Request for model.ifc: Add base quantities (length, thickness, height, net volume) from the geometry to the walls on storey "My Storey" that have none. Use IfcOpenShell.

First a look at what the model holds.

```python
import ifcopenshell
import ifcopenshell.util.element
import ifcopenshell.util.unit

model = ifcopenshell.open("model.ifc")
print(model.schema)
for unit_type in ("LENGTHUNIT", "AREAUNIT", "VOLUMEUNIT"):
    print(unit_type, ifcopenshell.util.unit.calculate_unit_scale(model, unit_type))
storey = next(s for s in model.by_type("IfcBuildingStorey") if s.Name == "My Storey")
walls = [e for e in ifcopenshell.util.element.get_decomposition(storey) if e.is_a("IfcWall")]
for e in sorted(walls, key=lambda e: e.id()):
    print(e.id(), e.is_a(), e.Name, list(ifcopenshell.util.element.get_psets(e, qtos_only=True)), sep=" | ")
```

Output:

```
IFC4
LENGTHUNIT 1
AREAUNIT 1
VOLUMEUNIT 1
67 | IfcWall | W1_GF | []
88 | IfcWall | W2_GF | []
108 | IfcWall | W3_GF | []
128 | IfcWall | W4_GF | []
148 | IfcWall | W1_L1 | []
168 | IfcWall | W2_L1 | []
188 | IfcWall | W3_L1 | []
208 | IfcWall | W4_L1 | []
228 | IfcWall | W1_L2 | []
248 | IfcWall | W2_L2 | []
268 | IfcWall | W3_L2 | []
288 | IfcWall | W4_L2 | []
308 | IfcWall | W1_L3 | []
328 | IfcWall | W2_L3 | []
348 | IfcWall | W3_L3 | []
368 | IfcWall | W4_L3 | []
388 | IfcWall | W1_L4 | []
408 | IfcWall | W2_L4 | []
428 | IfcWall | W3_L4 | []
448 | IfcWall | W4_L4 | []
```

```python
import ifcopenshell
import ifcopenshell.api.pset
import ifcopenshell.geom
import ifcopenshell.util.element
import ifcopenshell.util.shape
import ifcopenshell.util.unit

model = ifcopenshell.open("model.ifc")
unit_scale = ifcopenshell.util.unit.calculate_unit_scale(model)
volume_scale = ifcopenshell.util.unit.calculate_unit_scale(model, "VOLUMEUNIT")
settings = ifcopenshell.geom.settings()

storey = next(s for s in model.by_type("IfcBuildingStorey") if s.Name == "My Storey")
walls = [e for e in ifcopenshell.util.element.get_decomposition(storey) if e.is_a("IfcWall")]

for e in sorted(walls, key=lambda e: e.id()):
    if ifcopenshell.util.element.get_psets(e, qtos_only=True, should_inherit=False):
        continue
    # Geometry comes back in metres, in the element's own axes.
    shape = ifcopenshell.geom.create_shape(settings, e)
    values = {
        "Length": ifcopenshell.util.shape.get_x(shape.geometry) / unit_scale,
        "Width": ifcopenshell.util.shape.get_y(shape.geometry) / unit_scale,
        "Height": ifcopenshell.util.shape.get_z(shape.geometry) / unit_scale,
        "NetVolume": ifcopenshell.util.shape.get_volume(shape.geometry) / volume_scale,
    }
    qto = ifcopenshell.api.pset.add_qto(model, product=e, name="Qto_WallBaseQuantities")
    ifcopenshell.api.pset.edit_qto(model, qto=qto, properties=values)
    print(e.id(), {k: round(v, 3) for k, v in values.items()})

model.write("model_updated.ifc")
```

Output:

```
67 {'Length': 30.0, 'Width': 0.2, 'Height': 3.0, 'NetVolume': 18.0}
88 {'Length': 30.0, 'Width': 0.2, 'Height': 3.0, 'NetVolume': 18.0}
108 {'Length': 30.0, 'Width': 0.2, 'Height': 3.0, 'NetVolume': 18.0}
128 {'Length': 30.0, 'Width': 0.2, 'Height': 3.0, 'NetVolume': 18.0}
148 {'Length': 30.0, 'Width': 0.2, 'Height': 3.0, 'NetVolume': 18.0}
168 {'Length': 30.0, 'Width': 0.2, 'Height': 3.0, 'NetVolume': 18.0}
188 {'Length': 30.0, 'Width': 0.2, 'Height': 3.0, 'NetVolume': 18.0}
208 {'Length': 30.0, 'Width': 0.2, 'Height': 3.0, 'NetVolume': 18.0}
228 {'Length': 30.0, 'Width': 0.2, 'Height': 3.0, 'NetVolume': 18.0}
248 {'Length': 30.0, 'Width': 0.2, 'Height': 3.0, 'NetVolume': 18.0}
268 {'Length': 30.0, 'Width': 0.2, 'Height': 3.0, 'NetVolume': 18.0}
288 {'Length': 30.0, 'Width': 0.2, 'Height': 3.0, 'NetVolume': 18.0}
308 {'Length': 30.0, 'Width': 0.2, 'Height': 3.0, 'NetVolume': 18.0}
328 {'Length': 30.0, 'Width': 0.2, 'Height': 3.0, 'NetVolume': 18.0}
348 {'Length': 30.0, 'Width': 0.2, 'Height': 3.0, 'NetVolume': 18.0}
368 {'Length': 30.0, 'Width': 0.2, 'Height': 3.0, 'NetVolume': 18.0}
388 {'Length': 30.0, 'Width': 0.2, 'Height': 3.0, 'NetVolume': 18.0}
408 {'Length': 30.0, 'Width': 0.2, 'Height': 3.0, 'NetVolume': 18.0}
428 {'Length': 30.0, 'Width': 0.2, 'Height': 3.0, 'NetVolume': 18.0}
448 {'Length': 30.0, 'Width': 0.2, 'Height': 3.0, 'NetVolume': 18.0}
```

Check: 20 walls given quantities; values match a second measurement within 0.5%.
